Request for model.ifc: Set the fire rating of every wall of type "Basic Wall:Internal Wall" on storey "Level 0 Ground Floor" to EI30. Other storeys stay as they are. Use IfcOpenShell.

First a look at what the model holds.

```python
import ifcopenshell
import ifcopenshell.util.element

model = ifcopenshell.open("model.ifc")
print(model.schema)
storey = next(s for s in model.by_type("IfcBuildingStorey") if s.Name == "Level 0 Ground Floor")
walls = [e for e in ifcopenshell.util.element.get_decomposition(storey) if e.is_a("IfcWall")]
seen = {}
for e in walls:
    element_type = ifcopenshell.util.element.get_type(e)
    key = (element_type.Name if element_type != e and element_type else None, ifcopenshell.util.element.get_pset(e, "Pset_WallCommon", "FireRating"))
    seen[key] = seen.get(key, 0) + 1
for (name, value), count in sorted(seen.items(), key=str):
    print(count, "x", name, "|", value)
```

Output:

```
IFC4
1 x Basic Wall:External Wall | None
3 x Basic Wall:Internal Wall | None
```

```python
import ifcopenshell
import ifcopenshell.api.pset
import ifcopenshell.util.element

model = ifcopenshell.open("model.ifc")

storey = next(s for s in model.by_type("IfcBuildingStorey") if s.Name == "Level 0 Ground Floor")
walls = [e for e in ifcopenshell.util.element.get_decomposition(storey) if e.is_a("IfcWall")]

count = 0
for e in walls:
    element_type = ifcopenshell.util.element.get_type(e)
    if element_type in (None, e) or element_type.Name != "Basic Wall:Internal Wall":
        continue
    # add_pset returns the element's existing set when there is one.
    pset = ifcopenshell.api.pset.add_pset(model, product=e, name="Pset_WallCommon")
    ifcopenshell.api.pset.edit_pset(model, pset=pset, properties={"FireRating": "EI30"})
    count += 1

print(count, "walls updated")

model.write("model-out.ifc")
```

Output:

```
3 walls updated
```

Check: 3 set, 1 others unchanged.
